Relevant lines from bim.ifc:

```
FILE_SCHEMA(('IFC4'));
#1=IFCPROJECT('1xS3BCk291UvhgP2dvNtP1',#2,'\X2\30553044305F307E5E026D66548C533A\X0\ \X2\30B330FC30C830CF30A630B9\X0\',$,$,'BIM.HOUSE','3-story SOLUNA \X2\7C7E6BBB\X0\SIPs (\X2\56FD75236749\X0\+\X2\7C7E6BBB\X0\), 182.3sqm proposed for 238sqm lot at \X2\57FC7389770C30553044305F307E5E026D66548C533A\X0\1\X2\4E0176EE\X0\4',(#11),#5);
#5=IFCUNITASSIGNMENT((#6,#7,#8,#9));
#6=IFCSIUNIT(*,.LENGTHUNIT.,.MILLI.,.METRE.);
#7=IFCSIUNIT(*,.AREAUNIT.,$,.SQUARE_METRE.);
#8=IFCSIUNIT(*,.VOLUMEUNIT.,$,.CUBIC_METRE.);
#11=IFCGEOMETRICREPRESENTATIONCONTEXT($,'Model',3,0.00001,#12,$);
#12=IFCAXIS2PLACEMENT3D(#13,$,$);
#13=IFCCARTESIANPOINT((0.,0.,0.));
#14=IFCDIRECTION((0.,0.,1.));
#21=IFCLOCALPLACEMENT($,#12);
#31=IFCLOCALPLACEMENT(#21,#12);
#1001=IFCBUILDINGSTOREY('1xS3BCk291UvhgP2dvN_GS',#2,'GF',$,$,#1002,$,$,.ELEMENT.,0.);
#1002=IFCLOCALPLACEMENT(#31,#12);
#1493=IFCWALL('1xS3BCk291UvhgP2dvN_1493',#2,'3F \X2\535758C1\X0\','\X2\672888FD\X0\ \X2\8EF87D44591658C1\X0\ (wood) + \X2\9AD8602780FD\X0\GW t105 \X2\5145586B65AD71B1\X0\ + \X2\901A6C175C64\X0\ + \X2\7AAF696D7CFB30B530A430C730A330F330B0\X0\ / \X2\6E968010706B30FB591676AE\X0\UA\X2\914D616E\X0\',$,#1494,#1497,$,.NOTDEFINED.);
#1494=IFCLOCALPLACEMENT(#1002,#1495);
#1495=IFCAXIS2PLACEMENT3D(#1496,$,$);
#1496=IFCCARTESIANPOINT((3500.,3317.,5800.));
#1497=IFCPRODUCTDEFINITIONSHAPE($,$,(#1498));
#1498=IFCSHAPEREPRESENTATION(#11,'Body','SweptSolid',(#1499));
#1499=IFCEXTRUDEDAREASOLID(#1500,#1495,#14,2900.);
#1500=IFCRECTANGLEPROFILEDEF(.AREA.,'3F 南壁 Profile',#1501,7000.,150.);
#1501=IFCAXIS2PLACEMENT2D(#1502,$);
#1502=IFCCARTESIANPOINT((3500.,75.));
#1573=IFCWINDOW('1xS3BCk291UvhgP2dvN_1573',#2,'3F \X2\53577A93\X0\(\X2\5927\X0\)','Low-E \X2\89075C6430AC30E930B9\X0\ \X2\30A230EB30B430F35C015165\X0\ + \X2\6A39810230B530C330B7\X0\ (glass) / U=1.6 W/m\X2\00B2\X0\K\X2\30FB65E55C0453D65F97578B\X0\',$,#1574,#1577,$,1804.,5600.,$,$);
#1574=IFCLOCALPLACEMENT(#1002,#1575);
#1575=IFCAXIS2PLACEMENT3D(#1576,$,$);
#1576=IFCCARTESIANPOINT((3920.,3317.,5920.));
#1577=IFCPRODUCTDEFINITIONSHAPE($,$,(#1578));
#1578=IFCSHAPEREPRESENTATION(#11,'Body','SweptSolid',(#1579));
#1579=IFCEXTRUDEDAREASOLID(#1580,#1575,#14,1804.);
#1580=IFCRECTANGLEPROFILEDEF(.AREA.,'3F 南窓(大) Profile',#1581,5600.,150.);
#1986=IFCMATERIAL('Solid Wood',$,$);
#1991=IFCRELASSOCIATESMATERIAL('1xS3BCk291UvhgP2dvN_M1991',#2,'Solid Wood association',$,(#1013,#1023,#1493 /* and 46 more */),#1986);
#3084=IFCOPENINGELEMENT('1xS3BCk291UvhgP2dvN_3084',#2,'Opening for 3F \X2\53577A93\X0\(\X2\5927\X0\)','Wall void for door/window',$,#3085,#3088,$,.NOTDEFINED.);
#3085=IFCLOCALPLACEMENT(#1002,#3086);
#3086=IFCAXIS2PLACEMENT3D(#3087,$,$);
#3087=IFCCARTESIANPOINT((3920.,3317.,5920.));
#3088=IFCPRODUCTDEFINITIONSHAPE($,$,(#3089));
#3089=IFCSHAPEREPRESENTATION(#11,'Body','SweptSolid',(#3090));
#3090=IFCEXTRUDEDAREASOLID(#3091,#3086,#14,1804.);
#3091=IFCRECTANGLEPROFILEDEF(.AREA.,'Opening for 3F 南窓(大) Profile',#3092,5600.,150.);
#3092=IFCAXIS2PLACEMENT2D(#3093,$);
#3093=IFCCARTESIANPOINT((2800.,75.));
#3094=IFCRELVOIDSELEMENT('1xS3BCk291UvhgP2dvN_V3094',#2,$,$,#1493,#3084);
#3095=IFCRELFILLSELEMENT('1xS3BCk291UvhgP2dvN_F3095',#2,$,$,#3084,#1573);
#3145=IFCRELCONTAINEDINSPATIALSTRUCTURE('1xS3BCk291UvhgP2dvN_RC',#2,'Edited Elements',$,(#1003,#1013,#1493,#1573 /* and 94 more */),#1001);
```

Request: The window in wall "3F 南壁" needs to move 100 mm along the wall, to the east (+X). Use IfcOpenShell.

```python
import ifcopenshell
import ifcopenshell.api.geometry
import ifcopenshell.util.placement
import ifcopenshell.util.unit

model = ifcopenshell.open("bim.ifc")
unit_scale = ifcopenshell.util.unit.calculate_unit_scale(model)

window = model.by_guid("1xS3BCk291UvhgP2dvN_1573")
opening = window.FillsVoids[0].RelatingOpeningElement
wall = opening.VoidsElements[0].RelatingBuildingElement

wall_matrix = ifcopenshell.util.placement.get_local_placement(wall.ObjectPlacement)
shift = wall_matrix[:3, 0] * 0.1 / unit_scale
before = ifcopenshell.util.placement.get_local_placement(window.ObjectPlacement)[:3, 3].copy()

# The window is not placed relative to its opening, so move both.
for product in (opening, window):
    matrix = ifcopenshell.util.placement.get_local_placement(product.ObjectPlacement)
    matrix[:3, 3] += shift
    ifcopenshell.api.geometry.edit_object_placement(model, product=product, matrix=matrix, is_si=False)

after = ifcopenshell.util.placement.get_local_placement(window.ObjectPlacement)[:3, 3]
print("window moved by", (after - before).round(3) + 0.0)

model.write("bim-out.ifc")
```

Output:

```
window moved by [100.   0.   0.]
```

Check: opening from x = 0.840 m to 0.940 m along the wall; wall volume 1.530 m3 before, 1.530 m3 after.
